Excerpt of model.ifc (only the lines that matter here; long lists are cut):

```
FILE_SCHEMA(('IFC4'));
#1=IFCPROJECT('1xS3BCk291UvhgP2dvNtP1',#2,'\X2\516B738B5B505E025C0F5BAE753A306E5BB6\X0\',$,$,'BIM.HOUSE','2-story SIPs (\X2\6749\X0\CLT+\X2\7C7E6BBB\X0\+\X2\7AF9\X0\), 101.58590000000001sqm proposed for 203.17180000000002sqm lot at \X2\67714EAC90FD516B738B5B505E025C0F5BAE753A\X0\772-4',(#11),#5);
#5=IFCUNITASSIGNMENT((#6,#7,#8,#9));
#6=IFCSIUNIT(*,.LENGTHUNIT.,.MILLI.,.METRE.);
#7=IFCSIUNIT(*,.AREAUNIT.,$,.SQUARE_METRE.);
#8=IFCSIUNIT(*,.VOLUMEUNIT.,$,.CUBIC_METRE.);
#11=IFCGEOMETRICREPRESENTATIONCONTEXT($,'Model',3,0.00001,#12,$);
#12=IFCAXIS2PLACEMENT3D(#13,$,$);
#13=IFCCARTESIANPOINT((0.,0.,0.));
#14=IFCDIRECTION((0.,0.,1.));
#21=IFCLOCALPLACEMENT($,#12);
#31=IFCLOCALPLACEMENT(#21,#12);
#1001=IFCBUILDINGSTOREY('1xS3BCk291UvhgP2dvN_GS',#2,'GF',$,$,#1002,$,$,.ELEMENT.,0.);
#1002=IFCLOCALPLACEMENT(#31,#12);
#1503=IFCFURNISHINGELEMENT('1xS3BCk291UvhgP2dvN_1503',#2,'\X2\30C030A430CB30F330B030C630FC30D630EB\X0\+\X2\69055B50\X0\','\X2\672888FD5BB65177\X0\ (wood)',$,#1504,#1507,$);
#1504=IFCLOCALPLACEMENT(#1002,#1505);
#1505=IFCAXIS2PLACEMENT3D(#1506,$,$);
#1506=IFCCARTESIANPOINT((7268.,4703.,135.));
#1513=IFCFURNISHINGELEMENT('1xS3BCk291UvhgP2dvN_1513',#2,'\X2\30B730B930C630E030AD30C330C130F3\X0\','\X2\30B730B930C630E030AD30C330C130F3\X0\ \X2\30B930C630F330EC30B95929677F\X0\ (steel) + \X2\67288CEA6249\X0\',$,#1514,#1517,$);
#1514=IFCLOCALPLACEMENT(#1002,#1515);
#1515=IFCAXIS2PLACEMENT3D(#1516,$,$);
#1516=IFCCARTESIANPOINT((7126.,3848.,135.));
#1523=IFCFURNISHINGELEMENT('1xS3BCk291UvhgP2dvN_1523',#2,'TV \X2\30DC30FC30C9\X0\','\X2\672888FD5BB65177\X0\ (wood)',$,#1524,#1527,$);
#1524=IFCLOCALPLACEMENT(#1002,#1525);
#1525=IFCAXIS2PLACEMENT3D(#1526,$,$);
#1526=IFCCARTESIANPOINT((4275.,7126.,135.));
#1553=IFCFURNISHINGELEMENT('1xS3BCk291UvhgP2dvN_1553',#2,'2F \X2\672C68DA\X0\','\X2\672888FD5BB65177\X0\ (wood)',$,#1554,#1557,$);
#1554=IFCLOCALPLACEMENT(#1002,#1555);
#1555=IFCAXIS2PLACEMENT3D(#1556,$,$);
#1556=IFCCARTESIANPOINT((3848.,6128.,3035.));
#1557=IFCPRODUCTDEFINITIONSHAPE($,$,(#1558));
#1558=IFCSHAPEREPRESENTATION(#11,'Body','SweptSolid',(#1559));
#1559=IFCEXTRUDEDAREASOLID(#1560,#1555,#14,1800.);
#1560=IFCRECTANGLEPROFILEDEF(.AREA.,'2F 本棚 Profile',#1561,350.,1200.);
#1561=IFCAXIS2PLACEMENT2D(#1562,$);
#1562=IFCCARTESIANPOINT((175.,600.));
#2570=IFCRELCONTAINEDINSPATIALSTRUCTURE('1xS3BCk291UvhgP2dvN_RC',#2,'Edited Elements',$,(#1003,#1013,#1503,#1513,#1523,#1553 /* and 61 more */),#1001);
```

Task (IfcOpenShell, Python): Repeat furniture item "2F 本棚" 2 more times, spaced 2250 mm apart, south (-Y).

```python
import numpy as np
import ifcopenshell
import ifcopenshell.api.geometry
import ifcopenshell.api.root
import ifcopenshell.util.element
import ifcopenshell.util.placement

model = ifcopenshell.open("model.ifc")


def reuse_history(source, copy):
    """copy_class also copies each property set's owner history, people and application; keep the originals."""
    for rel in copy.IsDefinedBy:
        if rel.is_a("IfcRelDefinesByProperties") and (history := rel.RelatingPropertyDefinition.OwnerHistory):
            rel.RelatingPropertyDefinition.OwnerHistory = source.OwnerHistory
            ifcopenshell.util.element.remove_deep2(model, history)


source = model.by_guid("1xS3BCk291UvhgP2dvN_1553")
base = ifcopenshell.util.placement.get_local_placement(source.ObjectPlacement)
step = np.array([0.0, -1.0, 0.0]) * 2250.0

for i in range(1, 3):
    copy = ifcopenshell.api.root.copy_class(model, product=source)
    copy.Representation = ifcopenshell.util.element.copy_deep(
        model, source.Representation, exclude=["IfcGeometricRepresentationContext", "IfcRepresentationMap"]
    )
    reuse_history(source, copy)
    matrix = base.copy()
    matrix[:3, 3] += i * step
    print("added at", matrix[:3, 3].round(3) + 0.0)
    ifcopenshell.api.geometry.edit_object_placement(model, product=copy, matrix=matrix, is_si=False)

model.write("model_v2.ifc")
```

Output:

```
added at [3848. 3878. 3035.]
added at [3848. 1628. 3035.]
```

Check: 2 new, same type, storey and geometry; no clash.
